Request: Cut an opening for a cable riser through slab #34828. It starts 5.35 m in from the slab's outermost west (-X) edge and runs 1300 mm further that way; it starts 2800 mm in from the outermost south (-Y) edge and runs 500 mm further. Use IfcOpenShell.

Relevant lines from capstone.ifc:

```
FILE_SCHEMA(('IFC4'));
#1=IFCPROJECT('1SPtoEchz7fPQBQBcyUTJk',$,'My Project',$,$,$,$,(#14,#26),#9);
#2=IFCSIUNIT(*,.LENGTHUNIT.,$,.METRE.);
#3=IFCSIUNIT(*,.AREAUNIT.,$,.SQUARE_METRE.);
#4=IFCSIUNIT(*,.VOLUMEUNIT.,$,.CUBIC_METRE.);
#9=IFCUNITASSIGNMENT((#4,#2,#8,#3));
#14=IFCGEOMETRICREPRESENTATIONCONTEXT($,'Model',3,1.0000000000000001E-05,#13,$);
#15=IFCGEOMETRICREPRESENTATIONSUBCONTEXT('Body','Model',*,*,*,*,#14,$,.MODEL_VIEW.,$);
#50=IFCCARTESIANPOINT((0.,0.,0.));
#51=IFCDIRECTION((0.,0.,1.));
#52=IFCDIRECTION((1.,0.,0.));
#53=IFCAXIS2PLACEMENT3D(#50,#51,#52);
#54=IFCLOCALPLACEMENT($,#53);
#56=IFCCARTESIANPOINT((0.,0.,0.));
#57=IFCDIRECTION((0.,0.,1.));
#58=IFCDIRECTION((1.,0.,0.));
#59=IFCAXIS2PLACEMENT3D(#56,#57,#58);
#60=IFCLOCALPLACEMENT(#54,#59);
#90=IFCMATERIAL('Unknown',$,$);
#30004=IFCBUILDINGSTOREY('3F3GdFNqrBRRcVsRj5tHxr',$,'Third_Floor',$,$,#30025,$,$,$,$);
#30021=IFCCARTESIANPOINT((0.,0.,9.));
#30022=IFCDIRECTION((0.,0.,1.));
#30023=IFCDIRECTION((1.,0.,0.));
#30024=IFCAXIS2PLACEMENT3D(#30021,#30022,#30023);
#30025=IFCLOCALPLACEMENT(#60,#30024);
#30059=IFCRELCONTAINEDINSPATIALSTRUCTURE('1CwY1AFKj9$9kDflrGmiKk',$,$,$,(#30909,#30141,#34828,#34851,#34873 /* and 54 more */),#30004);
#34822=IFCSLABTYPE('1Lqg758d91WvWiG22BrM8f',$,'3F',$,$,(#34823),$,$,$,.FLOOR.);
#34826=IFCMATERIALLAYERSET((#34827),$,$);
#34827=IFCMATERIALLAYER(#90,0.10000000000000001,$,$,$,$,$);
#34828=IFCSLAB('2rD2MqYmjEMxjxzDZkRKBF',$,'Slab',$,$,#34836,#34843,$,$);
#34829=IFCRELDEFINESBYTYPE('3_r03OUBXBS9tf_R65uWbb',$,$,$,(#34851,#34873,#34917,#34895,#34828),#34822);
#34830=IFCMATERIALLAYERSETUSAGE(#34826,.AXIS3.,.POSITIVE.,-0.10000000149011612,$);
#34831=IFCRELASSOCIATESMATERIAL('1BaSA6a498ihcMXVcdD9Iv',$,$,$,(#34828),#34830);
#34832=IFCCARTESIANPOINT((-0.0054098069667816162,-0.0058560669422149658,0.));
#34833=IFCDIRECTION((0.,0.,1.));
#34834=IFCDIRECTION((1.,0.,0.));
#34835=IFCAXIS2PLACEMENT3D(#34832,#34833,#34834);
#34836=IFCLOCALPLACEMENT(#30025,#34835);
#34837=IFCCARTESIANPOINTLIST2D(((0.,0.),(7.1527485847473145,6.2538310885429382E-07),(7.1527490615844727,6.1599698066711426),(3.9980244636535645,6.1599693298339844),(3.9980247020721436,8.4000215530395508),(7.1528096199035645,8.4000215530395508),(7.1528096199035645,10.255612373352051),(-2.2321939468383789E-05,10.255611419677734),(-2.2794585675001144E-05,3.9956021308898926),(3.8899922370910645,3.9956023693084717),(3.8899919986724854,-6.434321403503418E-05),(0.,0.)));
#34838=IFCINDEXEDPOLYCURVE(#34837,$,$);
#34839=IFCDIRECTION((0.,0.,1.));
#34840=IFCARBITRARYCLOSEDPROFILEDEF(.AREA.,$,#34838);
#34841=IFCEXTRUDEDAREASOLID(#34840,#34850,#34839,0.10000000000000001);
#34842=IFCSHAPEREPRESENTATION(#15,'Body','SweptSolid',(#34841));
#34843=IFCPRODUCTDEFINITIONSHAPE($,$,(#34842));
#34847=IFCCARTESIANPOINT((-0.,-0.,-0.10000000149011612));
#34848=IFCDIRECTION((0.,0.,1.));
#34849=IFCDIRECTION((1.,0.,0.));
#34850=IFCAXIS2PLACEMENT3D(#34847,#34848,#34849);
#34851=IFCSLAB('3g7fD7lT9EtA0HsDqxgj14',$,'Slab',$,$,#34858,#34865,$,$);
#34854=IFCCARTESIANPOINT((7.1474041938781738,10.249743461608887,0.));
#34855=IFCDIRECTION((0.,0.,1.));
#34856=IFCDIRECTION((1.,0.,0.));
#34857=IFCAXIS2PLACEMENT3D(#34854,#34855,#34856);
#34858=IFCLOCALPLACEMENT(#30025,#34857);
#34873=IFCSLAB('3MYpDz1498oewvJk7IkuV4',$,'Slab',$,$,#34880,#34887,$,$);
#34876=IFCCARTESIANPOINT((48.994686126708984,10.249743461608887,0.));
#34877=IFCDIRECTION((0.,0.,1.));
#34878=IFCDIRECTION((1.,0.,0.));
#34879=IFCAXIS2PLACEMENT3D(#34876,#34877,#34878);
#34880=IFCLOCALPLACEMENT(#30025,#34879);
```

```python
import numpy as np
import ifcopenshell
import ifcopenshell.api.feature
import ifcopenshell.api.geometry
import ifcopenshell.api.root
import ifcopenshell.geom
import ifcopenshell.util.placement
import ifcopenshell.util.representation
import ifcopenshell.util.shape
import ifcopenshell.util.unit

model = ifcopenshell.open("capstone.ifc")
unit_scale = ifcopenshell.util.unit.calculate_unit_scale(model)
settings = ifcopenshell.geom.settings()


def volume(element):
    """Net volume in cubic metres, openings subtracted."""
    shape = ifcopenshell.geom.create_shape(settings, element)
    return ifcopenshell.util.shape.get_volume(shape.geometry)


slab = model.by_id(34828)
before = volume(slab)

# Extent in the slab's own axes, in metres. The edges named are its -X and -Y sides.
slab_shape = ifcopenshell.geom.create_shape(settings, slab)
vertices = ifcopenshell.util.shape.get_vertices(slab_shape.geometry)
x_min, y_min, bottom = vertices.min(axis=0)
top = vertices[:, 2].max()

opening = ifcopenshell.api.root.create_entity(model, ifc_class="IfcOpeningElement", name="Cable riser opening", predefined_type="OPENING")
context = ifcopenshell.util.representation.get_context(model, "Model", "Body", "MODEL_VIEW")
width, depth = 1.3, 0.5
outline = [(0.0, 0.0), (width, 0.0), (width, depth), (0.0, depth), (0.0, 0.0)]
# Overshoot both faces by 50 mm so the cut is clean.
shape = ifcopenshell.api.geometry.add_slab_representation(
    model, context=context, depth=top - bottom + 0.1, polyline=outline
)
ifcopenshell.api.geometry.assign_representation(model, product=opening, representation=shape)

matrix = ifcopenshell.util.placement.get_local_placement(slab.ObjectPlacement)
matrix[:, 3] = matrix @ np.append(np.array([x_min + 5.35, y_min + 2.8, bottom - 0.05]) / unit_scale, 1.0)
ifcopenshell.api.geometry.edit_object_placement(model, product=opening, matrix=matrix, is_si=False)
ifcopenshell.api.feature.add_feature(model, feature=opening, element=slab)

after = volume(slab)

print(f"slab volume {before:.3f} -> {after:.3f} m3")

model.write("capstone-out.ifc")
```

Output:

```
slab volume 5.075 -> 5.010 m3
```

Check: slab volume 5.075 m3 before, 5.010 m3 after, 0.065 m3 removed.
